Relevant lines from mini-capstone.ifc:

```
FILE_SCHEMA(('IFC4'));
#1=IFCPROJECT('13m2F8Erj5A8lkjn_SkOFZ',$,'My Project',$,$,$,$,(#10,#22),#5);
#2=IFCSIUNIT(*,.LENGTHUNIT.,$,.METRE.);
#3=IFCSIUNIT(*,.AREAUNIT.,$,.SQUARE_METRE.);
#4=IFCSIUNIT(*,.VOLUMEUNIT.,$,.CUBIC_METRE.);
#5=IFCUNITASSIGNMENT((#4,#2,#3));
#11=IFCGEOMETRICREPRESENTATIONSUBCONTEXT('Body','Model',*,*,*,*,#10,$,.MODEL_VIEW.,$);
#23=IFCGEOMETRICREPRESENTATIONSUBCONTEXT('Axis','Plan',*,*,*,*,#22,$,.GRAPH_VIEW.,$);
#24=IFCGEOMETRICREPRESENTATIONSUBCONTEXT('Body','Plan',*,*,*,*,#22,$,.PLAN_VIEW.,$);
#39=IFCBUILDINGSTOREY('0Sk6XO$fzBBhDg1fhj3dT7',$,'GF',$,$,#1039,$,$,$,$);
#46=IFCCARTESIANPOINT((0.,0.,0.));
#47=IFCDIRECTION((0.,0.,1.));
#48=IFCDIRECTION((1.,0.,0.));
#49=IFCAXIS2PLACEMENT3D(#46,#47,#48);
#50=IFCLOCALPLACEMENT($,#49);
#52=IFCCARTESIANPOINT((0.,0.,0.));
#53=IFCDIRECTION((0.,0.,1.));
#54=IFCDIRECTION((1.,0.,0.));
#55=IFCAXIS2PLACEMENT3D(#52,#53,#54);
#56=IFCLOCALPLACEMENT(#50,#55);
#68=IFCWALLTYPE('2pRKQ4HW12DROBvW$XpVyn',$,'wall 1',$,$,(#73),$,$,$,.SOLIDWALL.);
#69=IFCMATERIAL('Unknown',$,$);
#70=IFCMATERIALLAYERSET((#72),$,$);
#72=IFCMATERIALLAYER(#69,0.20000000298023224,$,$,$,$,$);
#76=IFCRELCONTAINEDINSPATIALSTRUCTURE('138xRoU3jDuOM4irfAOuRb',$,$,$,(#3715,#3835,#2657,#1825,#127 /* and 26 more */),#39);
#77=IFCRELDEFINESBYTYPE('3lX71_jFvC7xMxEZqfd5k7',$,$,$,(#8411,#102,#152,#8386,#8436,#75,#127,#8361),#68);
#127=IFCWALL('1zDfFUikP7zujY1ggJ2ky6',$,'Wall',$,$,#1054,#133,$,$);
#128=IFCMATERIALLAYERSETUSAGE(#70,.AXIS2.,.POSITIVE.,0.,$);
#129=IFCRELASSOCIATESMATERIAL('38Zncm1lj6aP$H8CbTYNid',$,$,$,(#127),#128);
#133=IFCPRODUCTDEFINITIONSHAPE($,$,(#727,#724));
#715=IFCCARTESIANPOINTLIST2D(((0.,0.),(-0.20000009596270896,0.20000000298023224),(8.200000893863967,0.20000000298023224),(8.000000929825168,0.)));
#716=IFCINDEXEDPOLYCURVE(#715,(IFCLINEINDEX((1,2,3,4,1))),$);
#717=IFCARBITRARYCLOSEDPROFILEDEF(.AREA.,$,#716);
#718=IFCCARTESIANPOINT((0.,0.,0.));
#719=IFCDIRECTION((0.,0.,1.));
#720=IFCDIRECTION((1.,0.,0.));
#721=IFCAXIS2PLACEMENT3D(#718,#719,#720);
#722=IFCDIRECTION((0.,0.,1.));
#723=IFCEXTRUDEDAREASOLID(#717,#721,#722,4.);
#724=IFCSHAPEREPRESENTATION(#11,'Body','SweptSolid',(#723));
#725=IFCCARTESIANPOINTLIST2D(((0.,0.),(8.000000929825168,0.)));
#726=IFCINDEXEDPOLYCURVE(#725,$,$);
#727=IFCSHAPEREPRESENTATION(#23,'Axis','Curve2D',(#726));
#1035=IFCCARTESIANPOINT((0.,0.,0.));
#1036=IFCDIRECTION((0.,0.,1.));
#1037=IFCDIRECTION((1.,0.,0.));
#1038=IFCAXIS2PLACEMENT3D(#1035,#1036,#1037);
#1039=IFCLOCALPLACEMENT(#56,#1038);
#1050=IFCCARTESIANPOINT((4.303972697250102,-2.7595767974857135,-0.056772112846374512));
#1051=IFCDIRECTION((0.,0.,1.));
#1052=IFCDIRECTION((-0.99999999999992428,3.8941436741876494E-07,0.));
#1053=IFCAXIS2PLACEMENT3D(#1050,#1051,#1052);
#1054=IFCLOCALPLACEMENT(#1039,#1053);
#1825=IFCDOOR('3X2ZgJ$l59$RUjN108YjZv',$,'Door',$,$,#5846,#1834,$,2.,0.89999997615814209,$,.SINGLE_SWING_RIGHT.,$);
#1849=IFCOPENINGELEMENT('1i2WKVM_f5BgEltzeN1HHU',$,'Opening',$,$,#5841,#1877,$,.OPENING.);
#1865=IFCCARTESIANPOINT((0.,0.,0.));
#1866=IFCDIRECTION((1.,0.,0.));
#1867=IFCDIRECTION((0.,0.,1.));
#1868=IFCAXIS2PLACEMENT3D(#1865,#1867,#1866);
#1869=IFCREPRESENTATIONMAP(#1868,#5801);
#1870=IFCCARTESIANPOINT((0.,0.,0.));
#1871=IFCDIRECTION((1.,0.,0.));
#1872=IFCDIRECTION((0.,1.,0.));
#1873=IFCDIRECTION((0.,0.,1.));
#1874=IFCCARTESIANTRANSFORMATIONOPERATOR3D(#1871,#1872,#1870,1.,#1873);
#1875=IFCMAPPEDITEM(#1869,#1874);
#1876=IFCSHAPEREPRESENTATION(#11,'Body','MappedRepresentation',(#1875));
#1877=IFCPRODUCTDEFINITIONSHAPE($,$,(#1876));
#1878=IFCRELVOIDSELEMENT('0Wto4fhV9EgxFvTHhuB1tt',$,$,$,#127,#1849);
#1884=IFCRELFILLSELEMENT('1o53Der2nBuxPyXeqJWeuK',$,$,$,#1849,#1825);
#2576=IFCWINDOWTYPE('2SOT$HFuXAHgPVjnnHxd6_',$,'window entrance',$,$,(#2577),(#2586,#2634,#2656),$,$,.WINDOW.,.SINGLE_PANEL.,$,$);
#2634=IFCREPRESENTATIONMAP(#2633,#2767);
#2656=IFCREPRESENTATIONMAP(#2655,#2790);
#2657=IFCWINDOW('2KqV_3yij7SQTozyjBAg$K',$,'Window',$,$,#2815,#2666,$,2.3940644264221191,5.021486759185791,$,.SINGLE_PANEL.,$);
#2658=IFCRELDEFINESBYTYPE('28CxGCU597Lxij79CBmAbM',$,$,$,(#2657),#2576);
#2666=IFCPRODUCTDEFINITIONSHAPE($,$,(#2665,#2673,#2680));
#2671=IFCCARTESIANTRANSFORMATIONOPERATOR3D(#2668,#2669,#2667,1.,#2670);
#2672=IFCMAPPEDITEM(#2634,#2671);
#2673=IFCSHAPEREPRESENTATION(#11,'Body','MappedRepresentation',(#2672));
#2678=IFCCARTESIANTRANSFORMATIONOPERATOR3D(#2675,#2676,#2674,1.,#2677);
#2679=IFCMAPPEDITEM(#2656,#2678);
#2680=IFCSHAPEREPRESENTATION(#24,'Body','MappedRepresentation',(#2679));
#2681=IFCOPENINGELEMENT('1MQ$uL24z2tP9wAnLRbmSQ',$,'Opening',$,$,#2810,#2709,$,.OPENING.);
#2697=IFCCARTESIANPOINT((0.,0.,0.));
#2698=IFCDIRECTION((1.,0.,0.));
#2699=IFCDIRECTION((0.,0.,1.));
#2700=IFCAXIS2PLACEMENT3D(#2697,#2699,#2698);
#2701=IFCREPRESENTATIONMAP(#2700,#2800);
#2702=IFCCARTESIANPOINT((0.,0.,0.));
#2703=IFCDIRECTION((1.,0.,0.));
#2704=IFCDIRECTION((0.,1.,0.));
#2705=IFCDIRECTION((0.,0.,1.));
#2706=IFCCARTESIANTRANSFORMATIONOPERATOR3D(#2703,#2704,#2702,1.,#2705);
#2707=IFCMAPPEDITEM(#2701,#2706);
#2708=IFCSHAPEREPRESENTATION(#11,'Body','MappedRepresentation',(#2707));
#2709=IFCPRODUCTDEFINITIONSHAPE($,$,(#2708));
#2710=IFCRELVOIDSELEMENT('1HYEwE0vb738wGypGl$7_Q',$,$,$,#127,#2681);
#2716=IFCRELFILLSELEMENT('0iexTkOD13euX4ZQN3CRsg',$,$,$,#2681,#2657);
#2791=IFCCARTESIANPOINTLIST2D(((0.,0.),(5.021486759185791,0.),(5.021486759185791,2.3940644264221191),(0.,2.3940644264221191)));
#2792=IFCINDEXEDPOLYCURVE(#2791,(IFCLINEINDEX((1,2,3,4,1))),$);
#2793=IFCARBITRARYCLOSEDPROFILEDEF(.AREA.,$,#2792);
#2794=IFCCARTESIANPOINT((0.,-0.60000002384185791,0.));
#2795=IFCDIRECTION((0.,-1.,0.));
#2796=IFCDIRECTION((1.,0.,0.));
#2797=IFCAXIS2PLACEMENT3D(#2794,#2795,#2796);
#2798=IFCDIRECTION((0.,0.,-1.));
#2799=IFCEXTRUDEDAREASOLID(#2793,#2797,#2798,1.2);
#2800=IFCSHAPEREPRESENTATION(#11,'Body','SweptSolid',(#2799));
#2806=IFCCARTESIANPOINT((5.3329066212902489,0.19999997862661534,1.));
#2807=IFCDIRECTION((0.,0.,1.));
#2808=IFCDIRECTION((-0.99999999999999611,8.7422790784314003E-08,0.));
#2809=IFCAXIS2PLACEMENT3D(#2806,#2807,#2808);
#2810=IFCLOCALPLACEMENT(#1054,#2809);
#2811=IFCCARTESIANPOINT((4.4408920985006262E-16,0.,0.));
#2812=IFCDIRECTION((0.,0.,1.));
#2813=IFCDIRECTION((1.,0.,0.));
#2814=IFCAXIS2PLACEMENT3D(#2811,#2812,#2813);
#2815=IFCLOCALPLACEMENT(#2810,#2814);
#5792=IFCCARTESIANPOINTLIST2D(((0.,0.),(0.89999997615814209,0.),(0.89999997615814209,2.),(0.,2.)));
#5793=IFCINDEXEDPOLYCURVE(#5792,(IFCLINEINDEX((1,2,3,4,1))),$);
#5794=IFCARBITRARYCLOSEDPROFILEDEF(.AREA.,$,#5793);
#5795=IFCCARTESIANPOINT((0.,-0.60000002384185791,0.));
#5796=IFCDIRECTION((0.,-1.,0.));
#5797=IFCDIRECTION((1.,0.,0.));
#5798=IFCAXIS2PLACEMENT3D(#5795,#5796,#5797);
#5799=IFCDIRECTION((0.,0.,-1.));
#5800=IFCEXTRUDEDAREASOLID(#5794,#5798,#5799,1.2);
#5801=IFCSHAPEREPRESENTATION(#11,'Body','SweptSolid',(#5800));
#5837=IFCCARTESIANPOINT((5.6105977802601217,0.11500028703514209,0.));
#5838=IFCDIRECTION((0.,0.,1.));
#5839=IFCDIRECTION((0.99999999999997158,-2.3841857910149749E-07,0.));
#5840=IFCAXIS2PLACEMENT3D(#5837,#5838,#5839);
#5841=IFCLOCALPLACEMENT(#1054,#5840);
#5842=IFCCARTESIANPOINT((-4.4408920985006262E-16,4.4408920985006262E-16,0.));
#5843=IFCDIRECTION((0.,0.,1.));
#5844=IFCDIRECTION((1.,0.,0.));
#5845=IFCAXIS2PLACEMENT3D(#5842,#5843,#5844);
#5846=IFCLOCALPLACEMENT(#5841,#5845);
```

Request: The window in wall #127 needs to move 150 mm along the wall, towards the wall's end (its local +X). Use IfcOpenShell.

```python
import ifcopenshell
import ifcopenshell.api.geometry
import ifcopenshell.util.placement

model = ifcopenshell.open("mini-capstone.ifc")

window = model.by_guid("2KqV_3yij7SQTozyjBAg$K")
opening = window.FillsVoids[0].RelatingOpeningElement
wall = opening.VoidsElements[0].RelatingBuildingElement

wall_matrix = ifcopenshell.util.placement.get_local_placement(wall.ObjectPlacement)
shift = wall_matrix[:3, 0] * 0.15
before = ifcopenshell.util.placement.get_local_placement(window.ObjectPlacement)[:3, 3].copy()

# The window is placed relative to its opening, so it follows when the opening moves.
matrix = ifcopenshell.util.placement.get_local_placement(opening.ObjectPlacement)
matrix[:3, 3] += shift
ifcopenshell.api.geometry.edit_object_placement(
    model, product=opening, matrix=matrix, is_si=False, should_transform_children=True
)

after = ifcopenshell.util.placement.get_local_placement(window.ObjectPlacement)[:3, 3]
print("window moved by", (after - before).round(3) + 0.0)

model.write("mini-capstone_edited.ifc")
```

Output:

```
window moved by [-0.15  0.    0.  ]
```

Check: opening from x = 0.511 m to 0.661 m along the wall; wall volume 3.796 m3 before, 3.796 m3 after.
